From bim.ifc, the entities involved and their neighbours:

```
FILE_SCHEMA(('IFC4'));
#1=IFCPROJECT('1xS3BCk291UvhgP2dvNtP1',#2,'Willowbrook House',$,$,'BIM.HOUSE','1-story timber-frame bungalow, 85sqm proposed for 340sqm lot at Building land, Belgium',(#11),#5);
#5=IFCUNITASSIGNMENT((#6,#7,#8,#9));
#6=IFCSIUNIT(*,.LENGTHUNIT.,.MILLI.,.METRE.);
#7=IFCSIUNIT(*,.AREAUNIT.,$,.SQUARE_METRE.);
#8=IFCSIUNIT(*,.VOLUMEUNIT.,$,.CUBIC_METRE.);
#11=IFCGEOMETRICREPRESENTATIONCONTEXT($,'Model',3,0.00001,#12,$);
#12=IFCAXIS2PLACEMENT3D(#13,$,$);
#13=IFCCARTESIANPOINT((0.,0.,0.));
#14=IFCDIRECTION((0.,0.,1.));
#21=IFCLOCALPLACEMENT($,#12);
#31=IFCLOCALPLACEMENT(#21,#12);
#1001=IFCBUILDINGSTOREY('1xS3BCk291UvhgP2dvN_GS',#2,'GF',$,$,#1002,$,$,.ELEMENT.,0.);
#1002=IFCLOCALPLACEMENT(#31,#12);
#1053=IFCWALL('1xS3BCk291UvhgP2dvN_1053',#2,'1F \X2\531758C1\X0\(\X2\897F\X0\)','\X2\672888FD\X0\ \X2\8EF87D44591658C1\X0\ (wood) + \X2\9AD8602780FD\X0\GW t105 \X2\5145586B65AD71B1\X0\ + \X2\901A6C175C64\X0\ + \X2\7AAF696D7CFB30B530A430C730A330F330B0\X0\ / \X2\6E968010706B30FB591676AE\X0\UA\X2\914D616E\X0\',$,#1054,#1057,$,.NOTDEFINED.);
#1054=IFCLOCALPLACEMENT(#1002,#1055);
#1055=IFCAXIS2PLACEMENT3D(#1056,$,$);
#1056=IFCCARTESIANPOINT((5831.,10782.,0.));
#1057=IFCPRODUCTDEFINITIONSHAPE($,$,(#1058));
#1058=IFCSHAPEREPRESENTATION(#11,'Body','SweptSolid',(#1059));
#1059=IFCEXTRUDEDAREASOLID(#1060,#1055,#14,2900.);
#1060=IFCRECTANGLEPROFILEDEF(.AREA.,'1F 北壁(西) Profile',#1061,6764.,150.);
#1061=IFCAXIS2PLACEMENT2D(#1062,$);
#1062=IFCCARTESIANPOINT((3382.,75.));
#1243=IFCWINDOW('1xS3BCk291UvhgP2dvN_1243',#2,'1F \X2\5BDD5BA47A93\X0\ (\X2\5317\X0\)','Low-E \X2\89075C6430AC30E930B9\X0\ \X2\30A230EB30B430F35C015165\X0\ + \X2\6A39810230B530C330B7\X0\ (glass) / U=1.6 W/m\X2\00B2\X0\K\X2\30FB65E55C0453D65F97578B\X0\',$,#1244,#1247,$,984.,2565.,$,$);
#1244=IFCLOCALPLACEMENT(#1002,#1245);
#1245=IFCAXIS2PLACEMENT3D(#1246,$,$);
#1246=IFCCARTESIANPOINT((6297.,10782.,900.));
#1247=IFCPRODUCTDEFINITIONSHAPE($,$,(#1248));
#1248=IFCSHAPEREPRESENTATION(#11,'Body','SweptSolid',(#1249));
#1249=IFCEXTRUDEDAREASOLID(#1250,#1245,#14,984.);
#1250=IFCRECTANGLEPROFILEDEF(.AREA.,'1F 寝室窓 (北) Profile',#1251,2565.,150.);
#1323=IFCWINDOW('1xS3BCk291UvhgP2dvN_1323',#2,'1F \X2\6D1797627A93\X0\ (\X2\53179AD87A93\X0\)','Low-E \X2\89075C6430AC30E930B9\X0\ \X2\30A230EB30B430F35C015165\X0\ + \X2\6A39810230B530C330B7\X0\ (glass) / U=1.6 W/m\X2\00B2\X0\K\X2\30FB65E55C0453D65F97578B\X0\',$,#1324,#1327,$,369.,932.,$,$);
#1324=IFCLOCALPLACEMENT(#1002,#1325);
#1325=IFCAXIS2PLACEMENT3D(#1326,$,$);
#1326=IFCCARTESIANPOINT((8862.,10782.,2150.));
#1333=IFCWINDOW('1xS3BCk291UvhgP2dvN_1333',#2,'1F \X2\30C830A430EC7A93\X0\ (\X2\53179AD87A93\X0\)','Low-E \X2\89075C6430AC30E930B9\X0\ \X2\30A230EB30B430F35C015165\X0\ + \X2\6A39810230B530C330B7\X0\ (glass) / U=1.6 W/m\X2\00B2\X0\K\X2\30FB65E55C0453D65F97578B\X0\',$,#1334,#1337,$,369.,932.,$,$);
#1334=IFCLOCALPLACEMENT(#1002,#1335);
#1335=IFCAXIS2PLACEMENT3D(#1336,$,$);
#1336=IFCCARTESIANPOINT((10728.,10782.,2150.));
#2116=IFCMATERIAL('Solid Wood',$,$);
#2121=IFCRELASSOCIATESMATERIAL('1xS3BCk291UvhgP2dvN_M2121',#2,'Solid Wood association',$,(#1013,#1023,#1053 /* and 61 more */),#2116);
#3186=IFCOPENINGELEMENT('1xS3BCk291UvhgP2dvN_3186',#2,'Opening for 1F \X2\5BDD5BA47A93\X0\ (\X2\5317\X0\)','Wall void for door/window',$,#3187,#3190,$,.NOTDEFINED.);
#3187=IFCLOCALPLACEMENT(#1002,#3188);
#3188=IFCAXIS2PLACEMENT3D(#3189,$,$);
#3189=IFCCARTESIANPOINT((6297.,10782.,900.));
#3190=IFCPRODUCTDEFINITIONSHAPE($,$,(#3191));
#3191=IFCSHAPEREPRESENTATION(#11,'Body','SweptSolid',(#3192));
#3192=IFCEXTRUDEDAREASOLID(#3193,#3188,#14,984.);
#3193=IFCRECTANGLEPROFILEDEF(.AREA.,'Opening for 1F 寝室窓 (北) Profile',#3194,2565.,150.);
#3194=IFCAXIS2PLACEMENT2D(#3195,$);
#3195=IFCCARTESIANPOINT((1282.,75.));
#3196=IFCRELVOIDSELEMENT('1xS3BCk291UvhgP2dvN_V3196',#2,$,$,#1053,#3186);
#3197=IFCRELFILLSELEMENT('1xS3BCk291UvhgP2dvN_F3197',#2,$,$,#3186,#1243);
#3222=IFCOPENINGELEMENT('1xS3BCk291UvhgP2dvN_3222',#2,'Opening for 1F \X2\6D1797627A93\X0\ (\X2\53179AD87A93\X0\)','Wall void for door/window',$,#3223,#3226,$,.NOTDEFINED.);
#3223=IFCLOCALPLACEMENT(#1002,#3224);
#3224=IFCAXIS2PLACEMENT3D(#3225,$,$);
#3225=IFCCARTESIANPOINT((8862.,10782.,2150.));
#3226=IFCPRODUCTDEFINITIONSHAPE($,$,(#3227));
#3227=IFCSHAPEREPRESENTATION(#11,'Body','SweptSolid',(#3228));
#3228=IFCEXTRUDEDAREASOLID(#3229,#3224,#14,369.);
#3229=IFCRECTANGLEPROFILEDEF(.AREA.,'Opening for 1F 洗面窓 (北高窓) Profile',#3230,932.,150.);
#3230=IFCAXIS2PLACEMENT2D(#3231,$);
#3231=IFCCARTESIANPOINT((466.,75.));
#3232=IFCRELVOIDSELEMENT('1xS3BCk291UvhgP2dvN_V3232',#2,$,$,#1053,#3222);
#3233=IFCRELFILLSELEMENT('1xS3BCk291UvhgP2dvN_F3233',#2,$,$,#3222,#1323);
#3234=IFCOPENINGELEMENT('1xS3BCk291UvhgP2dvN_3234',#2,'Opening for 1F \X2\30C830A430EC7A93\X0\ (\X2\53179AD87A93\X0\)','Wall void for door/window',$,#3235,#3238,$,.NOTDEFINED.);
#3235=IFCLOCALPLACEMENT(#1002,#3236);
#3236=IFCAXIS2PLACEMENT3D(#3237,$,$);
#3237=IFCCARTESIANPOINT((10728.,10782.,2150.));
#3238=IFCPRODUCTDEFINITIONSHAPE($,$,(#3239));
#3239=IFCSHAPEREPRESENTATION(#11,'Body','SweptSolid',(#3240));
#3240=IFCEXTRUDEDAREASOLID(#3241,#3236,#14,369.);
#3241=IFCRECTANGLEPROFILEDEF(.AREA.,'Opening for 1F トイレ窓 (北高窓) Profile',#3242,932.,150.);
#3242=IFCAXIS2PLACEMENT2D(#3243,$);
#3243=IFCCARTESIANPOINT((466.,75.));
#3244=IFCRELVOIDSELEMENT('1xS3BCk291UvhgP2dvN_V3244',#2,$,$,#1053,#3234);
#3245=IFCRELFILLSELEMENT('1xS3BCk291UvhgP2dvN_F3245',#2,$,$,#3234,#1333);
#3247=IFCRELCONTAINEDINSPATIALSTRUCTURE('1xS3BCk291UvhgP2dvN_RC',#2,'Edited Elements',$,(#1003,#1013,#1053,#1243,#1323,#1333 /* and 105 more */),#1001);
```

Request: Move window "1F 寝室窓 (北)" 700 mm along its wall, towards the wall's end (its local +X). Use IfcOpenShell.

```python
import ifcopenshell
import ifcopenshell.api.geometry
import ifcopenshell.util.placement

model = ifcopenshell.open("bim.ifc")

window = model.by_guid("1xS3BCk291UvhgP2dvN_1243")
opening = window.FillsVoids[0].RelatingOpeningElement
wall = opening.VoidsElements[0].RelatingBuildingElement

wall_matrix = ifcopenshell.util.placement.get_local_placement(wall.ObjectPlacement)
shift = wall_matrix[:3, 0] * 700.0
before = ifcopenshell.util.placement.get_local_placement(window.ObjectPlacement)[:3, 3].copy()

# The window is not placed relative to its opening, so move both.
for product in (opening, window):
    matrix = ifcopenshell.util.placement.get_local_placement(product.ObjectPlacement)
    matrix[:3, 3] += shift
    ifcopenshell.api.geometry.edit_object_placement(model, product=product, matrix=matrix, is_si=False)

after = ifcopenshell.util.placement.get_local_placement(window.ObjectPlacement)[:3, 3]
print("window moved by", (after - before).round(3) + 0.0)

model.write("bim-out.ifc")
```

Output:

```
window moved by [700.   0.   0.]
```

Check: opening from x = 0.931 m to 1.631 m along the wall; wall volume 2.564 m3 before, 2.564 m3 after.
